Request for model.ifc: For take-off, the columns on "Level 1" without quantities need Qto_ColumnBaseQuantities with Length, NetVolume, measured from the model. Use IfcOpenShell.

First a look at what the model holds.

```python
import ifcopenshell
import ifcopenshell.util.element
import ifcopenshell.util.unit

model = ifcopenshell.open("model.ifc")
print(model.schema)
for unit_type in ("LENGTHUNIT", "AREAUNIT", "VOLUMEUNIT"):
    print(unit_type, ifcopenshell.util.unit.calculate_unit_scale(model, unit_type))
storey = next(s for s in model.by_type("IfcBuildingStorey") if s.Name == "Level 1")
columns = [e for e in ifcopenshell.util.element.get_decomposition(storey) if e.is_a("IfcColumn")]
for e in sorted(columns, key=lambda e: e.id()):
    print(e.id(), e.is_a(), e.Name, list(ifcopenshell.util.element.get_psets(e, qtos_only=True)), sep=" | ")
```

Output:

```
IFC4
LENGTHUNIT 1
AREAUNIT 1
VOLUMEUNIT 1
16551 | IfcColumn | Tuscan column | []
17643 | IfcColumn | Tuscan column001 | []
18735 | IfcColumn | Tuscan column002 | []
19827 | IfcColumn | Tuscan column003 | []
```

```python
import ifcopenshell
import ifcopenshell.api.pset
import ifcopenshell.geom
import ifcopenshell.util.element
import ifcopenshell.util.shape
import ifcopenshell.util.unit

model = ifcopenshell.open("model.ifc")
unit_scale = ifcopenshell.util.unit.calculate_unit_scale(model)
volume_scale = ifcopenshell.util.unit.calculate_unit_scale(model, "VOLUMEUNIT")
settings = ifcopenshell.geom.settings()

storey = next(s for s in model.by_type("IfcBuildingStorey") if s.Name == "Level 1")
columns = [e for e in ifcopenshell.util.element.get_decomposition(storey) if e.is_a("IfcColumn")]

for e in sorted(columns, key=lambda e: e.id()):
    if ifcopenshell.util.element.get_psets(e, qtos_only=True, should_inherit=False):
        continue
    # Geometry comes back in metres, in the element's own axes.
    shape = ifcopenshell.geom.create_shape(settings, e)
    values = {
        "Length": ifcopenshell.util.shape.get_z(shape.geometry) / unit_scale,
        "NetVolume": ifcopenshell.util.shape.get_volume(shape.geometry) / volume_scale,
    }
    qto = ifcopenshell.api.pset.add_qto(model, product=e, name="Qto_ColumnBaseQuantities")
    ifcopenshell.api.pset.edit_qto(model, qto=qto, properties=values)
    print(e.id(), {k: round(v, 3) for k, v in values.items()})

model.write("model_updated.ifc")
```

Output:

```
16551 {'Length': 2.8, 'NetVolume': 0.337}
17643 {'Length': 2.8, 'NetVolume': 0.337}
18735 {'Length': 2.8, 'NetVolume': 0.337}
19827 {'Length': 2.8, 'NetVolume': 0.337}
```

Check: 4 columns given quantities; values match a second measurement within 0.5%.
